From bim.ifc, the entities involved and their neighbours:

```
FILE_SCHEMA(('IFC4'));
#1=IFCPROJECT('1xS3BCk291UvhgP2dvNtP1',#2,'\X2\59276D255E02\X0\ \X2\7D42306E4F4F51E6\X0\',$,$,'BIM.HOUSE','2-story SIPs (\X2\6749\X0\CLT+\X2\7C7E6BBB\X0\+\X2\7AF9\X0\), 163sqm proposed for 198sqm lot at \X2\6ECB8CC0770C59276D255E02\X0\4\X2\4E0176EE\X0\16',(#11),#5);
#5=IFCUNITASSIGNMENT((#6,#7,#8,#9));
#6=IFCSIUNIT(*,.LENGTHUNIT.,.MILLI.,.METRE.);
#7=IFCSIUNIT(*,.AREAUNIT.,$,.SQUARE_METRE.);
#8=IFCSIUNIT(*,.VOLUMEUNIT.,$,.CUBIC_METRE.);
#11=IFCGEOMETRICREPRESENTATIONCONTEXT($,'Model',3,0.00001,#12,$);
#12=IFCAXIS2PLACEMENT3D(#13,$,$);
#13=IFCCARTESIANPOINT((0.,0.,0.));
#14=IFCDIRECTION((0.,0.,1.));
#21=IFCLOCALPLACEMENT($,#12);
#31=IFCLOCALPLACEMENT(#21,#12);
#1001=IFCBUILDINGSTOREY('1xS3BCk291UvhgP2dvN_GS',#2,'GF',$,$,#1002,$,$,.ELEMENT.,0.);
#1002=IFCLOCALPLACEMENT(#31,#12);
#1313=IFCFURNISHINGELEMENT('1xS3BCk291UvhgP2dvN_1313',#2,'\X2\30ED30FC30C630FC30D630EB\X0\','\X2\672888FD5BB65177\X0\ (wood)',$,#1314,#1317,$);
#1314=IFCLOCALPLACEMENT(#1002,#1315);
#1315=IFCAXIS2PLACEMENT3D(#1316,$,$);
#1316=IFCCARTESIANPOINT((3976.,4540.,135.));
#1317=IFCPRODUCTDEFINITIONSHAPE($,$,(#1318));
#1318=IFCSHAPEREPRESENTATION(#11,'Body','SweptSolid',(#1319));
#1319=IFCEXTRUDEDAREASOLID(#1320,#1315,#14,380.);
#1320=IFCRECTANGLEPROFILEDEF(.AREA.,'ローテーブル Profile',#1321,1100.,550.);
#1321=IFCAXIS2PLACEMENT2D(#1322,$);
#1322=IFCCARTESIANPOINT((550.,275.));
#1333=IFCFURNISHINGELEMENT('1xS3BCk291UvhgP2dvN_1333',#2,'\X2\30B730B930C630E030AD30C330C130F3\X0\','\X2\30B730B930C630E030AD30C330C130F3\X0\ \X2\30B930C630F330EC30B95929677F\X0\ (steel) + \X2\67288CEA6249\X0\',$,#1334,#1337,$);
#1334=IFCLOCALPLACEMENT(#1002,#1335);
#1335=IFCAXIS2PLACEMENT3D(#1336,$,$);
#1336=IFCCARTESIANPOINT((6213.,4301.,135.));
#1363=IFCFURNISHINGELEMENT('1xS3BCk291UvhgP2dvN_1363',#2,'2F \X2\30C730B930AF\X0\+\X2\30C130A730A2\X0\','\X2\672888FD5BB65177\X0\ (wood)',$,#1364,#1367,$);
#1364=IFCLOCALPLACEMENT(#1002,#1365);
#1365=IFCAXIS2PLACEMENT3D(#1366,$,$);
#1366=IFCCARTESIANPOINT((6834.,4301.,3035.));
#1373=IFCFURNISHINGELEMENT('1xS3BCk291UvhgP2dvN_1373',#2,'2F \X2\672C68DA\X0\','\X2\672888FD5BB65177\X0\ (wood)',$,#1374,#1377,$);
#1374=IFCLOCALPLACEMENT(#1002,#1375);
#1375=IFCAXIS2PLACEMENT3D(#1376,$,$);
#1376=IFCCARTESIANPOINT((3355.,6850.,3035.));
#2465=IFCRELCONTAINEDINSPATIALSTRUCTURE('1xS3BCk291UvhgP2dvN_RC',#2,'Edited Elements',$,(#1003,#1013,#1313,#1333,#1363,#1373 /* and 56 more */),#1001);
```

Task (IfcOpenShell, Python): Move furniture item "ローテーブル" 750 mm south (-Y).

```python
import ifcopenshell
import ifcopenshell.api.geometry
import ifcopenshell.util.placement
import ifcopenshell.util.unit

model = ifcopenshell.open("bim.ifc")
unit_scale = ifcopenshell.util.unit.calculate_unit_scale(model)

item = model.by_guid("1xS3BCk291UvhgP2dvN_1313")
matrix = ifcopenshell.util.placement.get_local_placement(item.ObjectPlacement)
matrix[1, 3] -= 0.75 / unit_scale
ifcopenshell.api.geometry.edit_object_placement(model, product=item, matrix=matrix, is_si=False)

print(ifcopenshell.util.placement.get_local_placement(item.ObjectPlacement).round(3) + 0.0)

model.write("bim_v2.ifc")
```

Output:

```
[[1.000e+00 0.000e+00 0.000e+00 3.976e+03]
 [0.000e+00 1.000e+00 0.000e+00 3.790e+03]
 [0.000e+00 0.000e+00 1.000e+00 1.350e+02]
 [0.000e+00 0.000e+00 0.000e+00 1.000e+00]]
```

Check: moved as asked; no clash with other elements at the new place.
